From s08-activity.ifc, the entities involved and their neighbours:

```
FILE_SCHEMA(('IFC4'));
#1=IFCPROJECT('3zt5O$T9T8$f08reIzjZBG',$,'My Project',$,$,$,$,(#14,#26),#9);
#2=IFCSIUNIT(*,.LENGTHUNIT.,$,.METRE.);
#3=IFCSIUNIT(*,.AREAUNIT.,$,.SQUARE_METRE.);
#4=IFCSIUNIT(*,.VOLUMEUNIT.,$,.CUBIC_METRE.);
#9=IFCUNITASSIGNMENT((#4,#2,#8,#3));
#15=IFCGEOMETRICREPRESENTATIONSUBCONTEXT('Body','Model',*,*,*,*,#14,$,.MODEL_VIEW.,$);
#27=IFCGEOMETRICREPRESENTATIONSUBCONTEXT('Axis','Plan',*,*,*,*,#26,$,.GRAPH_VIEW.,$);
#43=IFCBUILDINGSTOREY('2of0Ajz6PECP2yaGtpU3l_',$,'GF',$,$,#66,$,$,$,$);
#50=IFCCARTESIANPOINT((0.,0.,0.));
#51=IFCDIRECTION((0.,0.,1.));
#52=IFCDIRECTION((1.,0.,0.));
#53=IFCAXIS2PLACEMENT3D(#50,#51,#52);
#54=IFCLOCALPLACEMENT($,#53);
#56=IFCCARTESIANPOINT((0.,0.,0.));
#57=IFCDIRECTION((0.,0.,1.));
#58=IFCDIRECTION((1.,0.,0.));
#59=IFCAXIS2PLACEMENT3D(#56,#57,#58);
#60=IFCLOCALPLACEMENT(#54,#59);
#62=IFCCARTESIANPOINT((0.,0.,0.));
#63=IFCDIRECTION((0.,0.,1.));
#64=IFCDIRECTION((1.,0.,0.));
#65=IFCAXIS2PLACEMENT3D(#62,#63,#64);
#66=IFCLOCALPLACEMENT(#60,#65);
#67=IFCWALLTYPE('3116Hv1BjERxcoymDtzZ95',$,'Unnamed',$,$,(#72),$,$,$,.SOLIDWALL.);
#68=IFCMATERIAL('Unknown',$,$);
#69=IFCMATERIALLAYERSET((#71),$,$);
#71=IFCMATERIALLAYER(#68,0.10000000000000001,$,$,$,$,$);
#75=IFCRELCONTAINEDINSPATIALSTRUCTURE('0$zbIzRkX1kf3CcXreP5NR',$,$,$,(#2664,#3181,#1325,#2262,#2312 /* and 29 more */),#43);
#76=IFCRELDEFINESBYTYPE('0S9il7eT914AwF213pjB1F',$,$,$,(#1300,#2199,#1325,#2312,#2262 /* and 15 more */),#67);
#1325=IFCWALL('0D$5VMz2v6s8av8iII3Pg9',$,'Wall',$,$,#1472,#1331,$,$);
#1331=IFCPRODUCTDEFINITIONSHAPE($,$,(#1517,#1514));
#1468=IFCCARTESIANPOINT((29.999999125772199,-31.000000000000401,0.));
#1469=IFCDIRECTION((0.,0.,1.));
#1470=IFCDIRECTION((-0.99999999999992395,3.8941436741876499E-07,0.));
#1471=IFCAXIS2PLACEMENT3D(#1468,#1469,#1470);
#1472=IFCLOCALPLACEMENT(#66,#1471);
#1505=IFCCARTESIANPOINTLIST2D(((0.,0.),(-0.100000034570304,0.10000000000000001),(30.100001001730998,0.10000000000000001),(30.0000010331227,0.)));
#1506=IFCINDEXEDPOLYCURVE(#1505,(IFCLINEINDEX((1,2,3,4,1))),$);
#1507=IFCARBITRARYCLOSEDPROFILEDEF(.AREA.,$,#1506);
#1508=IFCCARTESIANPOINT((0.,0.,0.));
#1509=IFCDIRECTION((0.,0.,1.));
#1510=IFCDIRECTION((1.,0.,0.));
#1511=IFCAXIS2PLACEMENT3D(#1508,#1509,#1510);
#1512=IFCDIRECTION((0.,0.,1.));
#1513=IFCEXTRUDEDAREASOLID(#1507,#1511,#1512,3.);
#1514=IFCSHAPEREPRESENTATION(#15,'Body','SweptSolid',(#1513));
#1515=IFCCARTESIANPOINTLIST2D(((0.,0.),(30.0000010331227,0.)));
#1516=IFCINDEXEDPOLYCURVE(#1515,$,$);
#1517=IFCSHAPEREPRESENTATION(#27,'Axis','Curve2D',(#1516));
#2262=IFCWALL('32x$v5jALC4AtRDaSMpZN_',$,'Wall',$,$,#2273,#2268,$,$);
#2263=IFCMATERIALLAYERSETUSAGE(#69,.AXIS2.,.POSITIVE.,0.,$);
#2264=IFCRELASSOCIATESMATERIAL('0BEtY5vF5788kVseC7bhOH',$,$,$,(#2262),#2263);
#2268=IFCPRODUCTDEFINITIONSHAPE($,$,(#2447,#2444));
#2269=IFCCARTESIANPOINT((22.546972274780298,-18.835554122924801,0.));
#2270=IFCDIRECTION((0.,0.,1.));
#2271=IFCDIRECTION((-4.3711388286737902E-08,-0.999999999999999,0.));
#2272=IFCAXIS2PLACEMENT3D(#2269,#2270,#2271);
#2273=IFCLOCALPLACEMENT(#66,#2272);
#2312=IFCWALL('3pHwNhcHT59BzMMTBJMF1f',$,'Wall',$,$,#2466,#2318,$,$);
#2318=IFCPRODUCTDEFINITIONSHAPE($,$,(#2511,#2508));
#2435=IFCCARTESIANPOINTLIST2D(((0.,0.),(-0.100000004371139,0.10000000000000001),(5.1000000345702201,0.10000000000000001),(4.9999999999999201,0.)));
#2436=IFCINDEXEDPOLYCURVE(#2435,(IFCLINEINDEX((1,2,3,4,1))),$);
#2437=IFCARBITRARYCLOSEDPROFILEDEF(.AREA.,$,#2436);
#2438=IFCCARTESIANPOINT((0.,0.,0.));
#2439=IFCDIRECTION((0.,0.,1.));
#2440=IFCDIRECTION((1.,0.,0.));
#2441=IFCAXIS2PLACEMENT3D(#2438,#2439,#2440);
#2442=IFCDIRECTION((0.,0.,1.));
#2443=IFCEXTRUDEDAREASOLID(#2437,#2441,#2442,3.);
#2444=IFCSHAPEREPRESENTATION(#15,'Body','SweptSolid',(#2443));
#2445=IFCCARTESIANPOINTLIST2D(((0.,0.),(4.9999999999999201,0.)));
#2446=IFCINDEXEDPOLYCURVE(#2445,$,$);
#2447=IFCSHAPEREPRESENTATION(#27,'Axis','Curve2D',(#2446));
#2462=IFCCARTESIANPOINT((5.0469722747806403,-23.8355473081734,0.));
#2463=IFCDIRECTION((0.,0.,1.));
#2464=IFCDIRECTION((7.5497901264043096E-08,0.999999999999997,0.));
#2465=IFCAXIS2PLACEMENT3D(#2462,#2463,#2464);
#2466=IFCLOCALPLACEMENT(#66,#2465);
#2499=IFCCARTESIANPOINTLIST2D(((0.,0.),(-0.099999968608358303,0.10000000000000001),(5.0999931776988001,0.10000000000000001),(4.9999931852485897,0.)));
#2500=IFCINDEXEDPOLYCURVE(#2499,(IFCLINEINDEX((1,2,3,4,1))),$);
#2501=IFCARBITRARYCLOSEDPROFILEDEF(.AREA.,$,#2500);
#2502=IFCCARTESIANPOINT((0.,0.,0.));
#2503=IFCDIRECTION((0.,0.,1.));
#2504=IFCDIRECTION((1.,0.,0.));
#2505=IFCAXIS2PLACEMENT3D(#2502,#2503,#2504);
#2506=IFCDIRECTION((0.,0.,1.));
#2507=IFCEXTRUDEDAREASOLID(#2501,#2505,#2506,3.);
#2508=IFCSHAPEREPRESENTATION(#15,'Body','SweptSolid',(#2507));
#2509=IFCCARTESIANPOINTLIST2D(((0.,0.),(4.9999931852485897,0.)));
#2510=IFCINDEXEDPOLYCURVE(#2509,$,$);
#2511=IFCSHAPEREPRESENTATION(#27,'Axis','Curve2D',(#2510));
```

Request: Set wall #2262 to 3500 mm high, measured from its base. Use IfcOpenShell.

```python
import ifcopenshell
import ifcopenshell.geom
import ifcopenshell.util.representation
import ifcopenshell.util.shape

model = ifcopenshell.open("s08-activity.ifc")
settings = ifcopenshell.geom.settings()


def volume(element):
    """Net volume in cubic metres, openings subtracted."""
    shape = ifcopenshell.geom.create_shape(settings, element)
    return ifcopenshell.util.shape.get_volume(shape.geometry)


wall = model.by_guid("32x$v5jALC4AtRDaSMpZN_")
before = volume(wall)

body = ifcopenshell.util.representation.get_representation(wall, "Model", "Body")
solid = body.Items[0]
old_height = solid.Depth
solid.Depth = 3.5
after = volume(wall)

print(f"height {old_height:g} -> {solid.Depth:g}, volume {before:.3f} -> {after:.3f} m3")

model.write("s08-activity_edited.ifc")
```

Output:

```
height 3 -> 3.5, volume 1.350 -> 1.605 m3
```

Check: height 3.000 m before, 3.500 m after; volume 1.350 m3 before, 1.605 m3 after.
